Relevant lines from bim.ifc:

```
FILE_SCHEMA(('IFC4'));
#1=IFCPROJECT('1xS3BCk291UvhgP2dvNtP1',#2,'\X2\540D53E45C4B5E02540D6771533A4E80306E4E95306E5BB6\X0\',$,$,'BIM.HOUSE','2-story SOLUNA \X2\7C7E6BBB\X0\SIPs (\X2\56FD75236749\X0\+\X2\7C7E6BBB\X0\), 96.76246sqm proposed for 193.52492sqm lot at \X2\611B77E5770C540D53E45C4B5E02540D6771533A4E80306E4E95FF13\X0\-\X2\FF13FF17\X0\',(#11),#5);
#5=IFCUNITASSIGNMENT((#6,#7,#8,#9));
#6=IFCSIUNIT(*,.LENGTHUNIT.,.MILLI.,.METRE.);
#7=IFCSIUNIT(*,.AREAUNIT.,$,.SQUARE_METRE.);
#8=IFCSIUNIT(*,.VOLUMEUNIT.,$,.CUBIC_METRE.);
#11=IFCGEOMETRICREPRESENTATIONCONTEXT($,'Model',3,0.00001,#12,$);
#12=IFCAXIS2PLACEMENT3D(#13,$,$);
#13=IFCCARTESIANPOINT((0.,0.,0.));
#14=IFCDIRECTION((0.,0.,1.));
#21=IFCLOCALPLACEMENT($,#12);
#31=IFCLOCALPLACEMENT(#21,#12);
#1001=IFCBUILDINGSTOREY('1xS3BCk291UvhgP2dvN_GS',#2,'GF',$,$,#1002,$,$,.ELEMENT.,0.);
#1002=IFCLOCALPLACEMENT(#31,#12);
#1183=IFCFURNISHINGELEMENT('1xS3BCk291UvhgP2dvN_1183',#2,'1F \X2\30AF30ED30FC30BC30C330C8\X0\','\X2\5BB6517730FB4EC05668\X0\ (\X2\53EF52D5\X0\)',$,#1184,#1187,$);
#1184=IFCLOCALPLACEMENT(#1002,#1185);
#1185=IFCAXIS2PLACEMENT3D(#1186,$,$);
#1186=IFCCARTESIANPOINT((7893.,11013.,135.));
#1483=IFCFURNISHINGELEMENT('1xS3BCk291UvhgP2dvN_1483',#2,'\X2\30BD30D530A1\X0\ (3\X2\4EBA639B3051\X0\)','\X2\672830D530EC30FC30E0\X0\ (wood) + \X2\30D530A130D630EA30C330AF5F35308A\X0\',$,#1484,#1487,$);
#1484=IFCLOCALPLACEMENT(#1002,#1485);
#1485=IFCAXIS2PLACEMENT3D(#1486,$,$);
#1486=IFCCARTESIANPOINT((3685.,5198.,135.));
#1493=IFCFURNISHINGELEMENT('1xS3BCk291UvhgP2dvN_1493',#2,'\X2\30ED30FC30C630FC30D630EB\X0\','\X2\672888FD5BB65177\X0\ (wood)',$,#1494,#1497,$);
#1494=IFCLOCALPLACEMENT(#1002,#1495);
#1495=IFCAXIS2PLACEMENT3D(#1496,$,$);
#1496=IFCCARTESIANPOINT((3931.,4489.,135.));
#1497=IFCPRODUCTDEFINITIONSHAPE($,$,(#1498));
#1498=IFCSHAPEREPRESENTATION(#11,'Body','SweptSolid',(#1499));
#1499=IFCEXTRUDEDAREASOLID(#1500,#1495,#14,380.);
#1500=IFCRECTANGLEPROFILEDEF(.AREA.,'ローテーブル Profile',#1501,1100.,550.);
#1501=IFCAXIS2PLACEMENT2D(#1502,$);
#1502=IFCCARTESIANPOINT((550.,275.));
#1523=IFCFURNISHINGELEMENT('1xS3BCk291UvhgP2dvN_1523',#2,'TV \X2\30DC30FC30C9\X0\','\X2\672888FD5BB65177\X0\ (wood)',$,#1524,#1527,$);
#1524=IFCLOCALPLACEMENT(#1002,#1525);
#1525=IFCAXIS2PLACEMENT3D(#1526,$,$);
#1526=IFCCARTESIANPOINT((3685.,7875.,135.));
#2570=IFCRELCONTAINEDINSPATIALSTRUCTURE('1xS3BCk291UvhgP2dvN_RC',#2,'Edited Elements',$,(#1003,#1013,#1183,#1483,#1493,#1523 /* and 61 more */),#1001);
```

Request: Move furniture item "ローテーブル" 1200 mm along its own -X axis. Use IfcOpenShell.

```python
import ifcopenshell
import ifcopenshell.api.geometry
import ifcopenshell.util.placement
import ifcopenshell.util.unit

model = ifcopenshell.open("bim.ifc")
unit_scale = ifcopenshell.util.unit.calculate_unit_scale(model)

item = model.by_id(1493)
matrix = ifcopenshell.util.placement.get_local_placement(item.ObjectPlacement)
matrix[:3, 3] -= matrix[:3, 0] * 1.2 / unit_scale
ifcopenshell.api.geometry.edit_object_placement(model, product=item, matrix=matrix, is_si=False)

print(ifcopenshell.util.placement.get_local_placement(item.ObjectPlacement).round(3) + 0.0)

model.write("bim_updated.ifc")
```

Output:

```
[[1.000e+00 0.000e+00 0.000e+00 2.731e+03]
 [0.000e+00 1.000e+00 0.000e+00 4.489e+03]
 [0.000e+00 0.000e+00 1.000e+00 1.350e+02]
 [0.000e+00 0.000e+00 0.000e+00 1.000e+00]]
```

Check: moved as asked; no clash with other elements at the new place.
